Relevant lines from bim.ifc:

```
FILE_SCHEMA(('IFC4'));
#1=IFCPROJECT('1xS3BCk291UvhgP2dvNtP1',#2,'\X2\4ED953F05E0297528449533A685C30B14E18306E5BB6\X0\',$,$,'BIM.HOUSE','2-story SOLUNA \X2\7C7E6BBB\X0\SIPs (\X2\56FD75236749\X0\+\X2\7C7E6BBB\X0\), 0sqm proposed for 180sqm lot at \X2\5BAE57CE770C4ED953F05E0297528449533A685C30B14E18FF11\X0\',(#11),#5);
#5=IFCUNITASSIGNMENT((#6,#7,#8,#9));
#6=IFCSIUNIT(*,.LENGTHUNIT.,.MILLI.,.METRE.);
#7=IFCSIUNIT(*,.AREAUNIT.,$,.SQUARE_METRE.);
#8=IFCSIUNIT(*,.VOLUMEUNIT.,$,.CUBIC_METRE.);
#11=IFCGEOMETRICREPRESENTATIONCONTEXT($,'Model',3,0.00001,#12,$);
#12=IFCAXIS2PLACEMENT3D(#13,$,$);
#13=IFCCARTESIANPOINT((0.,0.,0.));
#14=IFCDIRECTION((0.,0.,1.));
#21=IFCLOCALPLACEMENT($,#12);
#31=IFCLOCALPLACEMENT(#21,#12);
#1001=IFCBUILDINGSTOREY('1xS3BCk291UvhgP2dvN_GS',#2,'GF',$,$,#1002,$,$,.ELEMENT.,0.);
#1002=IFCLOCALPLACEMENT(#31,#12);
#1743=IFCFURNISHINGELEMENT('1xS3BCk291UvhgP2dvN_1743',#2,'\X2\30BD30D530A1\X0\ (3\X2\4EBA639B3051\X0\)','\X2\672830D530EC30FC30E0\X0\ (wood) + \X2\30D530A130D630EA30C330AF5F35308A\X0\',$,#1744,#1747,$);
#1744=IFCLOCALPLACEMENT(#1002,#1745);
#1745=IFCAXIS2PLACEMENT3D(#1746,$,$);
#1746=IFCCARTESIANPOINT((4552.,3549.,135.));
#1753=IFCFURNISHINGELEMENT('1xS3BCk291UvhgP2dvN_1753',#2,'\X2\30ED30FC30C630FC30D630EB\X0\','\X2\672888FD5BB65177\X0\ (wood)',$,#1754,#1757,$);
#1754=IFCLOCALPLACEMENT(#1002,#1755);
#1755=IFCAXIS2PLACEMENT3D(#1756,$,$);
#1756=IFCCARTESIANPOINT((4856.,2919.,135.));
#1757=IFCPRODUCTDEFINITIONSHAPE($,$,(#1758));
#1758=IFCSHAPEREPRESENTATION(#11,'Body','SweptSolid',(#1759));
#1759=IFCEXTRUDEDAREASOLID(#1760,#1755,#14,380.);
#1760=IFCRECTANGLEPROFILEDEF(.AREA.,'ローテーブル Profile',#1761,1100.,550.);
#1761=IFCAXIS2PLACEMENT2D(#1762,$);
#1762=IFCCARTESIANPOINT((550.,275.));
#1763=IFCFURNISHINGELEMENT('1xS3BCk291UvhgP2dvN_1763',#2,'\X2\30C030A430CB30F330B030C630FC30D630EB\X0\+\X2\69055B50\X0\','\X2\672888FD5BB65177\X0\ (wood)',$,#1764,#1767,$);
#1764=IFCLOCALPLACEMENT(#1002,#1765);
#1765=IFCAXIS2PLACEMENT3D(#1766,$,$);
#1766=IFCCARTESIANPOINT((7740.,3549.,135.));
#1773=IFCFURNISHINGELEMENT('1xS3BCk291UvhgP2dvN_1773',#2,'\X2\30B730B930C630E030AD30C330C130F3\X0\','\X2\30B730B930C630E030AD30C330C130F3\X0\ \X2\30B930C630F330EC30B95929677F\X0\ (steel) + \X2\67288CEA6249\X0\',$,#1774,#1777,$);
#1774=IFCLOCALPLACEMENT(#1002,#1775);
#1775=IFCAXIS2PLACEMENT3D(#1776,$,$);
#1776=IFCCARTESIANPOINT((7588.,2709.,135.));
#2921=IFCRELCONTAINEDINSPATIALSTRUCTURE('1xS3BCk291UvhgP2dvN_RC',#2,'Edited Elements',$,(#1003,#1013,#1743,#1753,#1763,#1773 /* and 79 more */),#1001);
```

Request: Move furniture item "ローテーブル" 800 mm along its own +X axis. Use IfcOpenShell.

```python
import ifcopenshell
import ifcopenshell.api.geometry
import ifcopenshell.util.placement
import ifcopenshell.util.unit

model = ifcopenshell.open("bim.ifc")
unit_scale = ifcopenshell.util.unit.calculate_unit_scale(model)

item = model.by_guid("1xS3BCk291UvhgP2dvN_1753")
matrix = ifcopenshell.util.placement.get_local_placement(item.ObjectPlacement)
matrix[:3, 3] += matrix[:3, 0] * 0.8 / unit_scale
ifcopenshell.api.geometry.edit_object_placement(model, product=item, matrix=matrix, is_si=False)

print(ifcopenshell.util.placement.get_local_placement(item.ObjectPlacement).round(3) + 0.0)

model.write("bim-out.ifc")
```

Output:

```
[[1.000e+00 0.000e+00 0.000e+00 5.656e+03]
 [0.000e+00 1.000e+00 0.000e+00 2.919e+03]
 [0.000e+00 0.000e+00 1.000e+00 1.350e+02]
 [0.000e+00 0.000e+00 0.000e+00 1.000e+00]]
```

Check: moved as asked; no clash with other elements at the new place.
